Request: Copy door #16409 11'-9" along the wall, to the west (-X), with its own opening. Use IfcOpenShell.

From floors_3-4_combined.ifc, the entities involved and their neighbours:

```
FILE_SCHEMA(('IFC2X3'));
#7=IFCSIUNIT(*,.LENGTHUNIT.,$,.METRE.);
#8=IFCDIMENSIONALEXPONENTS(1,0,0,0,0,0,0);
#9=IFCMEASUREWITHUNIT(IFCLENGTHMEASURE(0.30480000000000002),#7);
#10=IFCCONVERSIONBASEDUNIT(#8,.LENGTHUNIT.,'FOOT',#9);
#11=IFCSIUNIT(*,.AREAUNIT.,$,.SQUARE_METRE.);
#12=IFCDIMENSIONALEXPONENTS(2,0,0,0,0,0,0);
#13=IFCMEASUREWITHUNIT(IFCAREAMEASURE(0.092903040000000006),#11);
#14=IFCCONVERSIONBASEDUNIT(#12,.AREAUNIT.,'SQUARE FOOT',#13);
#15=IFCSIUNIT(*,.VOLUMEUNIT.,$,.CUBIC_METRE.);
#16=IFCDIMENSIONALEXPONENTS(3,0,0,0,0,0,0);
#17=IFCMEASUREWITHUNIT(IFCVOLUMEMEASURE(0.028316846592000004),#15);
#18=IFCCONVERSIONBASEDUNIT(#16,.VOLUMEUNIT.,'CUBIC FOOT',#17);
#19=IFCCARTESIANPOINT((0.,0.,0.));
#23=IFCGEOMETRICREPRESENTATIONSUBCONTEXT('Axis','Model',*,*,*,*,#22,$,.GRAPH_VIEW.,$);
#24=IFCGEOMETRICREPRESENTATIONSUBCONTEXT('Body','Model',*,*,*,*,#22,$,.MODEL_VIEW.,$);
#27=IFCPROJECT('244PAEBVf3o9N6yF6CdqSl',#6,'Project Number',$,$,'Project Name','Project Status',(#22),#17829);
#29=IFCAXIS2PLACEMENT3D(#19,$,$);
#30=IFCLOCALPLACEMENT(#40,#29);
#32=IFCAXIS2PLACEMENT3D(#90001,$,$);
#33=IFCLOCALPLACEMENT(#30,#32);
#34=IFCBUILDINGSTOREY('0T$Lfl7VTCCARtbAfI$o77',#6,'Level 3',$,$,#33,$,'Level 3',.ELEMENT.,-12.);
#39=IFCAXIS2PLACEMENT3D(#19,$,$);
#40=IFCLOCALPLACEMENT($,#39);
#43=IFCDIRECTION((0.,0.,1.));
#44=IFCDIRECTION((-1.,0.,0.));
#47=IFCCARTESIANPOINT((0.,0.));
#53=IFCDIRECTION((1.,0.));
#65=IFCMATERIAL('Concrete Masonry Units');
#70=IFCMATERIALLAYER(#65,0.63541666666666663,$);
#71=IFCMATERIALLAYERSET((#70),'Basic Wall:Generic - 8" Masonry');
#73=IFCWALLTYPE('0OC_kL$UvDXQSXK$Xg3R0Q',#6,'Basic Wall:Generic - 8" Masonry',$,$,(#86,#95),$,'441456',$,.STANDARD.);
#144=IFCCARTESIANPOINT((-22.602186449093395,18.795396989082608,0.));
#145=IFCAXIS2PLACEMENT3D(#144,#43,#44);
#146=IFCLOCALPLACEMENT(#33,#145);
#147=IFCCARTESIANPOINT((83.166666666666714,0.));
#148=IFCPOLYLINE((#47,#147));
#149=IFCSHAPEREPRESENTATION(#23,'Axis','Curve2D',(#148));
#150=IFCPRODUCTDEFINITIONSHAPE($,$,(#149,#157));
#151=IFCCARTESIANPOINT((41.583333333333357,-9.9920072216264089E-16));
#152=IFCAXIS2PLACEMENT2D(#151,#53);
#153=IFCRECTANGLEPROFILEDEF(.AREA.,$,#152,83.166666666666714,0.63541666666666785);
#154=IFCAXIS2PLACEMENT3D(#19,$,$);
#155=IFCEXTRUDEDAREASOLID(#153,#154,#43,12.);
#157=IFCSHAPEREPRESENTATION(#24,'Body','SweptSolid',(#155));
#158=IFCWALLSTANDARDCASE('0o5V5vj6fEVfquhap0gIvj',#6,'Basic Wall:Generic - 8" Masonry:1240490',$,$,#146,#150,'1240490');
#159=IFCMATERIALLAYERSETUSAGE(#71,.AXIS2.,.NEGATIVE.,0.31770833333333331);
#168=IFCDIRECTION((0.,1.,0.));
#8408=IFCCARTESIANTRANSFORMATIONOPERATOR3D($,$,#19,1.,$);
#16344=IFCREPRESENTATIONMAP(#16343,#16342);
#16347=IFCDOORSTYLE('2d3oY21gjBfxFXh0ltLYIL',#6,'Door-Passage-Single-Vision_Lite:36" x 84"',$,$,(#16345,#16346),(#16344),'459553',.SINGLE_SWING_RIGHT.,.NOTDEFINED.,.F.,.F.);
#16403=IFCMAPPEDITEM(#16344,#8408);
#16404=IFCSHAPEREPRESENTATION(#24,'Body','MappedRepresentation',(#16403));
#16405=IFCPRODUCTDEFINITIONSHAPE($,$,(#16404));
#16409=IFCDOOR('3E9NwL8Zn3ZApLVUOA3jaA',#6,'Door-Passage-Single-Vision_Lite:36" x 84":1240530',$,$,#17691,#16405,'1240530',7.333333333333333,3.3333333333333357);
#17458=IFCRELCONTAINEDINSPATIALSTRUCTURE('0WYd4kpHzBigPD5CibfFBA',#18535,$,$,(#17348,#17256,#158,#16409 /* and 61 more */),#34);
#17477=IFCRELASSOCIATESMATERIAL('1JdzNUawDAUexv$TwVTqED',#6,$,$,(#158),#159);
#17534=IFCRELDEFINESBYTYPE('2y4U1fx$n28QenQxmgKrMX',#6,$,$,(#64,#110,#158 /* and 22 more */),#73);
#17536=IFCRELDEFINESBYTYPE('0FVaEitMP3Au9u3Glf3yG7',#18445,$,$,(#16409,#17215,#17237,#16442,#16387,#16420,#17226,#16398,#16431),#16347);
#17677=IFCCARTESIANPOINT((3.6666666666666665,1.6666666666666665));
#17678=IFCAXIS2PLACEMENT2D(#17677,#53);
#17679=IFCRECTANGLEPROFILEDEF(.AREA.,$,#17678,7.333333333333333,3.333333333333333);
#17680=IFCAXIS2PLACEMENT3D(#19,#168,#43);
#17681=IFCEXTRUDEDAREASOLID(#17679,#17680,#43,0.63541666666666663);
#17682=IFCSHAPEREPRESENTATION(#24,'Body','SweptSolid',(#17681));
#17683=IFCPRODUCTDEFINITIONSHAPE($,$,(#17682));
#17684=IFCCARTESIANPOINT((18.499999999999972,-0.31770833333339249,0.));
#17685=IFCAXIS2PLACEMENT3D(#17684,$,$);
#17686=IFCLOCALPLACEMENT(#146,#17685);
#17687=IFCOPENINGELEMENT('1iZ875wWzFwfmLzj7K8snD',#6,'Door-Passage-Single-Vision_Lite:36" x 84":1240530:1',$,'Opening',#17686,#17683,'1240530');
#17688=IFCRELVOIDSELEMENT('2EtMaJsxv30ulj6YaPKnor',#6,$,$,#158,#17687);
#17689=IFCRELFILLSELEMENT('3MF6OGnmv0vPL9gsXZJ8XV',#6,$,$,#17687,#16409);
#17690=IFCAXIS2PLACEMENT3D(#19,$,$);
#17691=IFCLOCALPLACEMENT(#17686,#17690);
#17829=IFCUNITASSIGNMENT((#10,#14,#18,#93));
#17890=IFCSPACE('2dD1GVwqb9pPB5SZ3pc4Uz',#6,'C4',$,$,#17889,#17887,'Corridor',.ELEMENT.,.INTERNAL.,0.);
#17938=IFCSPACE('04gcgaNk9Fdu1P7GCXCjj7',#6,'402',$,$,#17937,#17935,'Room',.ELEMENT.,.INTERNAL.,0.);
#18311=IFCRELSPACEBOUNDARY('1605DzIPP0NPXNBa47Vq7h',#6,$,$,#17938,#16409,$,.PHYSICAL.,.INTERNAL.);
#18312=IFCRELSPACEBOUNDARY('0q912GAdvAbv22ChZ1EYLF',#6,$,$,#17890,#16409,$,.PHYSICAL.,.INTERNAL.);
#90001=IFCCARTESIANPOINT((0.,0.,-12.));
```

```python
import ifcopenshell
import ifcopenshell.api.feature
import ifcopenshell.api.geometry
import ifcopenshell.api.root
import ifcopenshell.geom
import ifcopenshell.util.element
import ifcopenshell.util.placement
import ifcopenshell.util.shape
import ifcopenshell.util.unit

model = ifcopenshell.open("floors_3-4_combined.ifc")
unit_scale = ifcopenshell.util.unit.calculate_unit_scale(model)
settings = ifcopenshell.geom.settings()


def volume(element):
    """Net volume in cubic metres, openings subtracted."""
    shape = ifcopenshell.geom.create_shape(settings, element)
    return ifcopenshell.util.shape.get_volume(shape.geometry)


def reuse_history(source, copy):
    """copy_class also copies each property set's owner history, people and application; keep the originals."""
    for rel in copy.IsDefinedBy:
        if rel.is_a("IfcRelDefinesByProperties") and (history := rel.RelatingPropertyDefinition.OwnerHistory):
            rel.RelatingPropertyDefinition.OwnerHistory = source.OwnerHistory
            ifcopenshell.util.element.remove_deep2(model, history)


door = model.by_guid("3E9NwL8Zn3ZApLVUOA3jaA")
opening = door.FillsVoids[0].RelatingOpeningElement
wall = opening.VoidsElements[0].RelatingBuildingElement
before = volume(wall)
shift = ifcopenshell.util.placement.get_local_placement(wall.ObjectPlacement)[:3, 0] * 141 * 0.0254 / unit_scale

# copy_class copies the void relationship, type, container and properties, but no geometry.
new_opening = ifcopenshell.api.root.copy_class(model, product=opening)
new_opening.Representation = ifcopenshell.util.element.copy_deep(
    model, opening.Representation, exclude=["IfcGeometricRepresentationContext", "IfcRepresentationMap"]
)
new_opening.Name = 'Door-Passage-Single-Vision_Lite:36" x 84"'
new_opening.Tag = None
new_door = ifcopenshell.api.root.copy_class(model, product=door)
new_door.Representation = ifcopenshell.util.element.copy_deep(
    model, door.Representation, exclude=["IfcGeometricRepresentationContext", "IfcRepresentationMap"]
)
new_door.Name = 'Door-Passage-Single-Vision_Lite:36" x 84"'
new_door.Tag = None
reuse_history(door, new_door)
fills = ifcopenshell.api.feature.add_filling(model, opening=new_opening, element=new_door)
fills.OwnerHistory = new_door.OwnerHistory  # required in IFC2X3

for old, new in ((opening, new_opening), (door, new_door)):
    matrix = ifcopenshell.util.placement.get_local_placement(old.ObjectPlacement)
    matrix[:3, 3] += shift
    ifcopenshell.api.geometry.edit_object_placement(model, product=new, matrix=matrix, is_si=False)

after = volume(wall)

print(f"wall volume {before:.3f} -> {after:.3f} m3")

model.write("floors_3-4_combined_rev.ifc")
```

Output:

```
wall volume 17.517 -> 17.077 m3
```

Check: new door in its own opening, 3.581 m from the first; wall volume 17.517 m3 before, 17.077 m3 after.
